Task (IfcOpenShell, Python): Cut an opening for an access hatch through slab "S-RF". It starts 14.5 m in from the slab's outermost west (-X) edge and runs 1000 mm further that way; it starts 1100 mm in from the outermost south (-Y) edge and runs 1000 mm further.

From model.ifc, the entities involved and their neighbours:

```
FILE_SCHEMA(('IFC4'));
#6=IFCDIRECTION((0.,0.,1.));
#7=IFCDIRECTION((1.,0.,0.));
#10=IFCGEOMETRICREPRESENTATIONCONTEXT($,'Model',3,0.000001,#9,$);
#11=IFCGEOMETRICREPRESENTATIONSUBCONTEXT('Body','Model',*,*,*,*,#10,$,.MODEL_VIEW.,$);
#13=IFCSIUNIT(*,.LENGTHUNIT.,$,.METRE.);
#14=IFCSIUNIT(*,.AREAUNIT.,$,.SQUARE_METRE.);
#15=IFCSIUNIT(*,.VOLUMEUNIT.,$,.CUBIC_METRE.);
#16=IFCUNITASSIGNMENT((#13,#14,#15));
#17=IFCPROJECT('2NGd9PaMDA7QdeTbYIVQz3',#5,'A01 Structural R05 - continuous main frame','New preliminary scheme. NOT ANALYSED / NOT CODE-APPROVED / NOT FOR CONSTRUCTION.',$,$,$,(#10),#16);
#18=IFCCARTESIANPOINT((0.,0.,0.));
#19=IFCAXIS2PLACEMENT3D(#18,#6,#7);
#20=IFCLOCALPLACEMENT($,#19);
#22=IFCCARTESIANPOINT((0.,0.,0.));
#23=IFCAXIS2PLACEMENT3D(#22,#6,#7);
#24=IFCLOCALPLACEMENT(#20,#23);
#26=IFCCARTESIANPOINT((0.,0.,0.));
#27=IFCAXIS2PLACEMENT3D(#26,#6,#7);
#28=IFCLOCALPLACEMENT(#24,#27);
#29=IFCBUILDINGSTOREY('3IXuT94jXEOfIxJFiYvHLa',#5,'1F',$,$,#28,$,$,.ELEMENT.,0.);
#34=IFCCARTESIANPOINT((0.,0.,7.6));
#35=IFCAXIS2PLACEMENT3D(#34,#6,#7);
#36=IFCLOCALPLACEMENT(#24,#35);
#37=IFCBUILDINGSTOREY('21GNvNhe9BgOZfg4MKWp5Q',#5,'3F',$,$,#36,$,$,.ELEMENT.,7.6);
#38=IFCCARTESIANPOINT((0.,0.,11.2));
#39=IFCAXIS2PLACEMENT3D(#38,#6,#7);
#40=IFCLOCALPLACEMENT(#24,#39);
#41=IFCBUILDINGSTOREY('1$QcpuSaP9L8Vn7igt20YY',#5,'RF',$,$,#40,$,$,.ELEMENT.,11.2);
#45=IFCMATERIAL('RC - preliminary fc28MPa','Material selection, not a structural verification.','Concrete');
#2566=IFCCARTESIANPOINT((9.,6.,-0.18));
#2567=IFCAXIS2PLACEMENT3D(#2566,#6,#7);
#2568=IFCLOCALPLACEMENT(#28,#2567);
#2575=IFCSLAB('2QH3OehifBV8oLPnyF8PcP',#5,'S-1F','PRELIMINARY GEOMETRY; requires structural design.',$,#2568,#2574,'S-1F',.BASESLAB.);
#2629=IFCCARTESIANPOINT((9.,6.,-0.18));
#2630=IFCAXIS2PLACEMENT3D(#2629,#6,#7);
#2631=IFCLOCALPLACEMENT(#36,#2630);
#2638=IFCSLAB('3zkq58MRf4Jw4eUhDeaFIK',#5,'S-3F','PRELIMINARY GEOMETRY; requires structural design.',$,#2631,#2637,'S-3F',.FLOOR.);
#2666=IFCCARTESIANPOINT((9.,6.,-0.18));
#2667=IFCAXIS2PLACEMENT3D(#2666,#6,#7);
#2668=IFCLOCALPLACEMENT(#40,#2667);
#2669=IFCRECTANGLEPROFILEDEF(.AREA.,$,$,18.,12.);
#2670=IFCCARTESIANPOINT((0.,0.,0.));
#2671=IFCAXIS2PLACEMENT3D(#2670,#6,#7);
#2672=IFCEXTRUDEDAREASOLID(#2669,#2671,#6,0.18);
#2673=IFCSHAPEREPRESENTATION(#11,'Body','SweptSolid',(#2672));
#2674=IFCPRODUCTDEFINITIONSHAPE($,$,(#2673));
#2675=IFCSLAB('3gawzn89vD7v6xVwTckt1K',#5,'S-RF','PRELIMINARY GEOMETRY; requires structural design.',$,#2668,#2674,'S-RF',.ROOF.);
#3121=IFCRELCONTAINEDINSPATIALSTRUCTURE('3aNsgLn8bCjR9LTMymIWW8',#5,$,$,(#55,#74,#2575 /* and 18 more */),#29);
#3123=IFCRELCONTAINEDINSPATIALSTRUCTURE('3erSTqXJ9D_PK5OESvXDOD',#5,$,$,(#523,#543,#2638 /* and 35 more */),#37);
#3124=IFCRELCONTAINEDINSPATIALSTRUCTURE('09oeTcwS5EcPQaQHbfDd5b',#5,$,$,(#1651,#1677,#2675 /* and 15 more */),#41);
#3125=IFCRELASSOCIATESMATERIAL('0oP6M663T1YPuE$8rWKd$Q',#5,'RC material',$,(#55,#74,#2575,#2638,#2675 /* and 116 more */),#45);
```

```python
import numpy as np
import ifcopenshell
import ifcopenshell.api.feature
import ifcopenshell.api.geometry
import ifcopenshell.api.root
import ifcopenshell.geom
import ifcopenshell.util.placement
import ifcopenshell.util.representation
import ifcopenshell.util.shape
import ifcopenshell.util.unit

model = ifcopenshell.open("model.ifc")
unit_scale = ifcopenshell.util.unit.calculate_unit_scale(model)
settings = ifcopenshell.geom.settings()


def volume(element):
    """Net volume in cubic metres, openings subtracted."""
    shape = ifcopenshell.geom.create_shape(settings, element)
    return ifcopenshell.util.shape.get_volume(shape.geometry)


slab = model.by_guid("3gawzn89vD7v6xVwTckt1K")
before = volume(slab)

# Extent in the slab's own axes, in metres. The edges named are its -X and -Y sides.
slab_shape = ifcopenshell.geom.create_shape(settings, slab)
vertices = ifcopenshell.util.shape.get_vertices(slab_shape.geometry)
x_min, y_min, bottom = vertices.min(axis=0)
top = vertices[:, 2].max()

opening = ifcopenshell.api.root.create_entity(model, ifc_class="IfcOpeningElement", name="Access hatch opening", predefined_type="OPENING")
context = ifcopenshell.util.representation.get_context(model, "Model", "Body", "MODEL_VIEW")
width, depth = 1, 1
outline = [(0.0, 0.0), (width, 0.0), (width, depth), (0.0, depth), (0.0, 0.0)]
# Overshoot both faces by 50 mm so the cut is clean.
shape = ifcopenshell.api.geometry.add_slab_representation(
    model, context=context, depth=top - bottom + 0.1, polyline=outline
)
ifcopenshell.api.geometry.assign_representation(model, product=opening, representation=shape)

matrix = ifcopenshell.util.placement.get_local_placement(slab.ObjectPlacement)
matrix[:, 3] = matrix @ np.append(np.array([x_min + 14.5, y_min + 1.1, bottom - 0.05]) / unit_scale, 1.0)
ifcopenshell.api.geometry.edit_object_placement(model, product=opening, matrix=matrix, is_si=False)
ifcopenshell.api.feature.add_feature(model, feature=opening, element=slab)

after = volume(slab)

print(f"slab volume {before:.3f} -> {after:.3f} m3")

model.write("model_edited.ifc")
```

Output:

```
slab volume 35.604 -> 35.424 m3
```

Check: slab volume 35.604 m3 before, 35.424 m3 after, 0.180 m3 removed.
